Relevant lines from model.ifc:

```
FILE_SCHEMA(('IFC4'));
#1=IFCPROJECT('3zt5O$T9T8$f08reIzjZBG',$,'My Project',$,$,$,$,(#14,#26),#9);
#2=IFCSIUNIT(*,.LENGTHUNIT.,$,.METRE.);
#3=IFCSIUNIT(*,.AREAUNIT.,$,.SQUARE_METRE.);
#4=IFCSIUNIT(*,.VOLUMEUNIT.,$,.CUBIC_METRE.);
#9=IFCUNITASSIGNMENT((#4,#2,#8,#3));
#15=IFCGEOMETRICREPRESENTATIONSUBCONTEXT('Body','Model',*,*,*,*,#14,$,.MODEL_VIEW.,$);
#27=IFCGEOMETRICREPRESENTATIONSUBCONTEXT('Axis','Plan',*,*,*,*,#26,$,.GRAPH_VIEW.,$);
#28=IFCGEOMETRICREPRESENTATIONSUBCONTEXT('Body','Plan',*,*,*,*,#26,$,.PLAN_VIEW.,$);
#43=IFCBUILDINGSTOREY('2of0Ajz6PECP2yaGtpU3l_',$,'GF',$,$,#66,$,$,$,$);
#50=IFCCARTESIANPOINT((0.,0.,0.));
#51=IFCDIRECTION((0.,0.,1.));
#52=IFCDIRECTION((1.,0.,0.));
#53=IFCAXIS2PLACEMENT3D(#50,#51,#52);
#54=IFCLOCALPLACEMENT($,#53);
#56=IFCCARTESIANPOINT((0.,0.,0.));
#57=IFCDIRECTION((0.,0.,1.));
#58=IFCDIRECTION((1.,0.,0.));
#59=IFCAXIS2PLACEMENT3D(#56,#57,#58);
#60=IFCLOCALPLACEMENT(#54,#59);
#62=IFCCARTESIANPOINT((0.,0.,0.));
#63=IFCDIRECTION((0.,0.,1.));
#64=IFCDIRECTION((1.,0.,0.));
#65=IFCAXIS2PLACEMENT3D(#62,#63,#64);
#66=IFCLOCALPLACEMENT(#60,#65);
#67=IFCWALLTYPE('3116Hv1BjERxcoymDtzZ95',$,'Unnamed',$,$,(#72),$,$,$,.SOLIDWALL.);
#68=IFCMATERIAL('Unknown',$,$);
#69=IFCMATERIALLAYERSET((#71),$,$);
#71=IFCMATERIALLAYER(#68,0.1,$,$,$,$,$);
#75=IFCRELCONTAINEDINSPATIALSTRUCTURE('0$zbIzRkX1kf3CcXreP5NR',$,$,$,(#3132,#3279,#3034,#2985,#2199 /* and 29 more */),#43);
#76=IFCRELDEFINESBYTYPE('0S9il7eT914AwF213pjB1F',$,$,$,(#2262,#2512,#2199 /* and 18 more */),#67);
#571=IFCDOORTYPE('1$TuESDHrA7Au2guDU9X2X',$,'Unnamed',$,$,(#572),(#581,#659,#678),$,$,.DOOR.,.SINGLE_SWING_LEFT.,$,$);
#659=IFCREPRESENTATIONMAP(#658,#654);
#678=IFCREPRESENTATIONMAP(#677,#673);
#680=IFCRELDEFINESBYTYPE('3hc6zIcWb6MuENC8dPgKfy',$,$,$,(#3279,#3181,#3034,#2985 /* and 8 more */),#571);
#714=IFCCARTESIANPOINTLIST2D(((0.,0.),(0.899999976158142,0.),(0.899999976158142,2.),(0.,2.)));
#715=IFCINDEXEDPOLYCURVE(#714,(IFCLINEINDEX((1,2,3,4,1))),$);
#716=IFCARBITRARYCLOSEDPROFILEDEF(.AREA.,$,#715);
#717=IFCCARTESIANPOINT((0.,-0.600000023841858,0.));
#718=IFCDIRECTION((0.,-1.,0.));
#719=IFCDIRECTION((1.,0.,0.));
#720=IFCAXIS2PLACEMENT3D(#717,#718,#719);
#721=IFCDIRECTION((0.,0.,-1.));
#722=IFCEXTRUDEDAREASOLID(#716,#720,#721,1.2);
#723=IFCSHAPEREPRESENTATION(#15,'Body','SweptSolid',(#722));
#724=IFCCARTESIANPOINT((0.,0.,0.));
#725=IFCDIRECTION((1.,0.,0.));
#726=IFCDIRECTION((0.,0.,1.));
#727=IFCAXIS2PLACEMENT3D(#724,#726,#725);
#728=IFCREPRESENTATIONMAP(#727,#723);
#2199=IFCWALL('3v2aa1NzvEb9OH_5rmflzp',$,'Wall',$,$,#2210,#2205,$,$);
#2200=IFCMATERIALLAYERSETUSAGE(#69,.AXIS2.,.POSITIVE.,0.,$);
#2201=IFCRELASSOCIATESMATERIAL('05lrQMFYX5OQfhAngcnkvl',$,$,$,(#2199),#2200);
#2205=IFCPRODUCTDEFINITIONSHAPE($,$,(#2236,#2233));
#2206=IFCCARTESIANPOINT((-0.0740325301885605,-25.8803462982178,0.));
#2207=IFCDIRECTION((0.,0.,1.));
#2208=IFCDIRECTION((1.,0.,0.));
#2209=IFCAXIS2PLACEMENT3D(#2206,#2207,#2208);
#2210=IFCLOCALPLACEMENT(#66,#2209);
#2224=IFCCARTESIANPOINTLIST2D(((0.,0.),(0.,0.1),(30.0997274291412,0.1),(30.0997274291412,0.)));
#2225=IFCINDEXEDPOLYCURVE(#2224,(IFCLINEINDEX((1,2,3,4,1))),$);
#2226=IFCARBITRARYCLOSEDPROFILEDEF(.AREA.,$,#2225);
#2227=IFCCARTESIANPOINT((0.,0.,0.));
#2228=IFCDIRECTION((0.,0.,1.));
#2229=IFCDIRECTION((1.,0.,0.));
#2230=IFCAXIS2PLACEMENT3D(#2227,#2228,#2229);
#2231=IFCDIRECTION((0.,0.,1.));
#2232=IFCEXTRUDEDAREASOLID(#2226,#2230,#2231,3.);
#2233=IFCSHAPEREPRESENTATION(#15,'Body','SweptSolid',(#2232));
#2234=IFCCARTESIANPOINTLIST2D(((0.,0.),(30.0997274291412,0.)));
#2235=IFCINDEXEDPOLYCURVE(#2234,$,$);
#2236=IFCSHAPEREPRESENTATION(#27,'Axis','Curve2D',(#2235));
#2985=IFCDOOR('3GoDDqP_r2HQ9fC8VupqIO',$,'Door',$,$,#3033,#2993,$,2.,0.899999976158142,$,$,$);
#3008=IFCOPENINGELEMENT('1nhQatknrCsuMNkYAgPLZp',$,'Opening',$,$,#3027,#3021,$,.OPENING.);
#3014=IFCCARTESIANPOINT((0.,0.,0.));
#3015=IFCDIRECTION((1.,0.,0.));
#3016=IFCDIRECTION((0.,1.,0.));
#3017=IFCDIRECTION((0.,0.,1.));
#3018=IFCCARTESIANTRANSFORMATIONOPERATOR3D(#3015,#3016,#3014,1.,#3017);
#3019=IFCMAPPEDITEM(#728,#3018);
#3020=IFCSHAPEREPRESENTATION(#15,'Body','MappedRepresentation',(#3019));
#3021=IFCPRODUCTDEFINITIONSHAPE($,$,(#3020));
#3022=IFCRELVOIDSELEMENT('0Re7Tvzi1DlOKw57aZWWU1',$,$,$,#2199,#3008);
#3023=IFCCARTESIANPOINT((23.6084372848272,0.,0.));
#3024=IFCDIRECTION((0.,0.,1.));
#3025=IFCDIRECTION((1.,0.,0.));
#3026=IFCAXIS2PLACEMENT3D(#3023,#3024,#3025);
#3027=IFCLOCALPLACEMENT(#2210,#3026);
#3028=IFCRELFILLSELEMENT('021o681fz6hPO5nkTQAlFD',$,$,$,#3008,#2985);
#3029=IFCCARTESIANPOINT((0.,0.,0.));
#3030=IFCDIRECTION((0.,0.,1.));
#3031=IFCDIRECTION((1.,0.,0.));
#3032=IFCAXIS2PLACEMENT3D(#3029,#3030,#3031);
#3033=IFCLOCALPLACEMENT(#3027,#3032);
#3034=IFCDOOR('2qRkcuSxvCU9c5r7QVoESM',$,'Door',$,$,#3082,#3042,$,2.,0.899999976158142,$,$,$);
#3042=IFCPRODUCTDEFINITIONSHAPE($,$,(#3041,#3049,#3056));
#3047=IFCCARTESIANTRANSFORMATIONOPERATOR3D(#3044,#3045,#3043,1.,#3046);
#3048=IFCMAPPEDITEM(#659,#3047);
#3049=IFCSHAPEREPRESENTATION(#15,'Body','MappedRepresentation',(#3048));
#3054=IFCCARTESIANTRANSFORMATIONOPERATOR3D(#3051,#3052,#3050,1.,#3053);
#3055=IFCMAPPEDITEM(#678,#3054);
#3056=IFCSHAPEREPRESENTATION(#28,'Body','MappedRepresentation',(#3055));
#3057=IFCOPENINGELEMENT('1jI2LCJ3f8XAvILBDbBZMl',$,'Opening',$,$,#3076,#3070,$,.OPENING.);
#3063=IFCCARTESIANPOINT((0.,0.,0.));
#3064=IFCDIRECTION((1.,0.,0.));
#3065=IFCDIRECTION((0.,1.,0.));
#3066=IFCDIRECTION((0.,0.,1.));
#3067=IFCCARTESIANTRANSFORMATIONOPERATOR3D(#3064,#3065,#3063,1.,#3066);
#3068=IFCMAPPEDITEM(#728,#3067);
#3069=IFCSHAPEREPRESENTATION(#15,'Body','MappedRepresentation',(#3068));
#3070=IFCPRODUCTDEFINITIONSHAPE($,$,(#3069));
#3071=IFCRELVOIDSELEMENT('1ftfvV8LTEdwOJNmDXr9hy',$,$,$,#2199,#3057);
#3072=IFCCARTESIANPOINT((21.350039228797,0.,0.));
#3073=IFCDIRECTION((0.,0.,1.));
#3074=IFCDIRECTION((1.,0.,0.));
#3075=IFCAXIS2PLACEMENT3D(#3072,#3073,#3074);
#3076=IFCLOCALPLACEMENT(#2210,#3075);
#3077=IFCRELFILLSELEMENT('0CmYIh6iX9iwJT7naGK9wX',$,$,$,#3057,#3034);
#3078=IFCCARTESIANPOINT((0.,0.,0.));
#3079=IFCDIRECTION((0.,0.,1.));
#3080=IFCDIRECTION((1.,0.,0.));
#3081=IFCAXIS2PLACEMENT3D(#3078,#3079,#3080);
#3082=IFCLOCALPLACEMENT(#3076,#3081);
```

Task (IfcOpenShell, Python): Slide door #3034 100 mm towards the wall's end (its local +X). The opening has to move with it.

```python
import ifcopenshell
import ifcopenshell.api.geometry
import ifcopenshell.util.placement

model = ifcopenshell.open("model.ifc")

door = model.by_guid("2qRkcuSxvCU9c5r7QVoESM")
opening = door.FillsVoids[0].RelatingOpeningElement
wall = opening.VoidsElements[0].RelatingBuildingElement

wall_matrix = ifcopenshell.util.placement.get_local_placement(wall.ObjectPlacement)
shift = wall_matrix[:3, 0] * 0.1
before = ifcopenshell.util.placement.get_local_placement(door.ObjectPlacement)[:3, 3].copy()

# The door is placed relative to its opening, so it follows when the opening moves.
matrix = ifcopenshell.util.placement.get_local_placement(opening.ObjectPlacement)
matrix[:3, 3] += shift
ifcopenshell.api.geometry.edit_object_placement(
    model, product=opening, matrix=matrix, is_si=False, should_transform_children=True
)

after = ifcopenshell.util.placement.get_local_placement(door.ObjectPlacement)[:3, 3]
print("door moved by", (after - before).round(3) + 0.0)

model.write("model_rev.ifc")
```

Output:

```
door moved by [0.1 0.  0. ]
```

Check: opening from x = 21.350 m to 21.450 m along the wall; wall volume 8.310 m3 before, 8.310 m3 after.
